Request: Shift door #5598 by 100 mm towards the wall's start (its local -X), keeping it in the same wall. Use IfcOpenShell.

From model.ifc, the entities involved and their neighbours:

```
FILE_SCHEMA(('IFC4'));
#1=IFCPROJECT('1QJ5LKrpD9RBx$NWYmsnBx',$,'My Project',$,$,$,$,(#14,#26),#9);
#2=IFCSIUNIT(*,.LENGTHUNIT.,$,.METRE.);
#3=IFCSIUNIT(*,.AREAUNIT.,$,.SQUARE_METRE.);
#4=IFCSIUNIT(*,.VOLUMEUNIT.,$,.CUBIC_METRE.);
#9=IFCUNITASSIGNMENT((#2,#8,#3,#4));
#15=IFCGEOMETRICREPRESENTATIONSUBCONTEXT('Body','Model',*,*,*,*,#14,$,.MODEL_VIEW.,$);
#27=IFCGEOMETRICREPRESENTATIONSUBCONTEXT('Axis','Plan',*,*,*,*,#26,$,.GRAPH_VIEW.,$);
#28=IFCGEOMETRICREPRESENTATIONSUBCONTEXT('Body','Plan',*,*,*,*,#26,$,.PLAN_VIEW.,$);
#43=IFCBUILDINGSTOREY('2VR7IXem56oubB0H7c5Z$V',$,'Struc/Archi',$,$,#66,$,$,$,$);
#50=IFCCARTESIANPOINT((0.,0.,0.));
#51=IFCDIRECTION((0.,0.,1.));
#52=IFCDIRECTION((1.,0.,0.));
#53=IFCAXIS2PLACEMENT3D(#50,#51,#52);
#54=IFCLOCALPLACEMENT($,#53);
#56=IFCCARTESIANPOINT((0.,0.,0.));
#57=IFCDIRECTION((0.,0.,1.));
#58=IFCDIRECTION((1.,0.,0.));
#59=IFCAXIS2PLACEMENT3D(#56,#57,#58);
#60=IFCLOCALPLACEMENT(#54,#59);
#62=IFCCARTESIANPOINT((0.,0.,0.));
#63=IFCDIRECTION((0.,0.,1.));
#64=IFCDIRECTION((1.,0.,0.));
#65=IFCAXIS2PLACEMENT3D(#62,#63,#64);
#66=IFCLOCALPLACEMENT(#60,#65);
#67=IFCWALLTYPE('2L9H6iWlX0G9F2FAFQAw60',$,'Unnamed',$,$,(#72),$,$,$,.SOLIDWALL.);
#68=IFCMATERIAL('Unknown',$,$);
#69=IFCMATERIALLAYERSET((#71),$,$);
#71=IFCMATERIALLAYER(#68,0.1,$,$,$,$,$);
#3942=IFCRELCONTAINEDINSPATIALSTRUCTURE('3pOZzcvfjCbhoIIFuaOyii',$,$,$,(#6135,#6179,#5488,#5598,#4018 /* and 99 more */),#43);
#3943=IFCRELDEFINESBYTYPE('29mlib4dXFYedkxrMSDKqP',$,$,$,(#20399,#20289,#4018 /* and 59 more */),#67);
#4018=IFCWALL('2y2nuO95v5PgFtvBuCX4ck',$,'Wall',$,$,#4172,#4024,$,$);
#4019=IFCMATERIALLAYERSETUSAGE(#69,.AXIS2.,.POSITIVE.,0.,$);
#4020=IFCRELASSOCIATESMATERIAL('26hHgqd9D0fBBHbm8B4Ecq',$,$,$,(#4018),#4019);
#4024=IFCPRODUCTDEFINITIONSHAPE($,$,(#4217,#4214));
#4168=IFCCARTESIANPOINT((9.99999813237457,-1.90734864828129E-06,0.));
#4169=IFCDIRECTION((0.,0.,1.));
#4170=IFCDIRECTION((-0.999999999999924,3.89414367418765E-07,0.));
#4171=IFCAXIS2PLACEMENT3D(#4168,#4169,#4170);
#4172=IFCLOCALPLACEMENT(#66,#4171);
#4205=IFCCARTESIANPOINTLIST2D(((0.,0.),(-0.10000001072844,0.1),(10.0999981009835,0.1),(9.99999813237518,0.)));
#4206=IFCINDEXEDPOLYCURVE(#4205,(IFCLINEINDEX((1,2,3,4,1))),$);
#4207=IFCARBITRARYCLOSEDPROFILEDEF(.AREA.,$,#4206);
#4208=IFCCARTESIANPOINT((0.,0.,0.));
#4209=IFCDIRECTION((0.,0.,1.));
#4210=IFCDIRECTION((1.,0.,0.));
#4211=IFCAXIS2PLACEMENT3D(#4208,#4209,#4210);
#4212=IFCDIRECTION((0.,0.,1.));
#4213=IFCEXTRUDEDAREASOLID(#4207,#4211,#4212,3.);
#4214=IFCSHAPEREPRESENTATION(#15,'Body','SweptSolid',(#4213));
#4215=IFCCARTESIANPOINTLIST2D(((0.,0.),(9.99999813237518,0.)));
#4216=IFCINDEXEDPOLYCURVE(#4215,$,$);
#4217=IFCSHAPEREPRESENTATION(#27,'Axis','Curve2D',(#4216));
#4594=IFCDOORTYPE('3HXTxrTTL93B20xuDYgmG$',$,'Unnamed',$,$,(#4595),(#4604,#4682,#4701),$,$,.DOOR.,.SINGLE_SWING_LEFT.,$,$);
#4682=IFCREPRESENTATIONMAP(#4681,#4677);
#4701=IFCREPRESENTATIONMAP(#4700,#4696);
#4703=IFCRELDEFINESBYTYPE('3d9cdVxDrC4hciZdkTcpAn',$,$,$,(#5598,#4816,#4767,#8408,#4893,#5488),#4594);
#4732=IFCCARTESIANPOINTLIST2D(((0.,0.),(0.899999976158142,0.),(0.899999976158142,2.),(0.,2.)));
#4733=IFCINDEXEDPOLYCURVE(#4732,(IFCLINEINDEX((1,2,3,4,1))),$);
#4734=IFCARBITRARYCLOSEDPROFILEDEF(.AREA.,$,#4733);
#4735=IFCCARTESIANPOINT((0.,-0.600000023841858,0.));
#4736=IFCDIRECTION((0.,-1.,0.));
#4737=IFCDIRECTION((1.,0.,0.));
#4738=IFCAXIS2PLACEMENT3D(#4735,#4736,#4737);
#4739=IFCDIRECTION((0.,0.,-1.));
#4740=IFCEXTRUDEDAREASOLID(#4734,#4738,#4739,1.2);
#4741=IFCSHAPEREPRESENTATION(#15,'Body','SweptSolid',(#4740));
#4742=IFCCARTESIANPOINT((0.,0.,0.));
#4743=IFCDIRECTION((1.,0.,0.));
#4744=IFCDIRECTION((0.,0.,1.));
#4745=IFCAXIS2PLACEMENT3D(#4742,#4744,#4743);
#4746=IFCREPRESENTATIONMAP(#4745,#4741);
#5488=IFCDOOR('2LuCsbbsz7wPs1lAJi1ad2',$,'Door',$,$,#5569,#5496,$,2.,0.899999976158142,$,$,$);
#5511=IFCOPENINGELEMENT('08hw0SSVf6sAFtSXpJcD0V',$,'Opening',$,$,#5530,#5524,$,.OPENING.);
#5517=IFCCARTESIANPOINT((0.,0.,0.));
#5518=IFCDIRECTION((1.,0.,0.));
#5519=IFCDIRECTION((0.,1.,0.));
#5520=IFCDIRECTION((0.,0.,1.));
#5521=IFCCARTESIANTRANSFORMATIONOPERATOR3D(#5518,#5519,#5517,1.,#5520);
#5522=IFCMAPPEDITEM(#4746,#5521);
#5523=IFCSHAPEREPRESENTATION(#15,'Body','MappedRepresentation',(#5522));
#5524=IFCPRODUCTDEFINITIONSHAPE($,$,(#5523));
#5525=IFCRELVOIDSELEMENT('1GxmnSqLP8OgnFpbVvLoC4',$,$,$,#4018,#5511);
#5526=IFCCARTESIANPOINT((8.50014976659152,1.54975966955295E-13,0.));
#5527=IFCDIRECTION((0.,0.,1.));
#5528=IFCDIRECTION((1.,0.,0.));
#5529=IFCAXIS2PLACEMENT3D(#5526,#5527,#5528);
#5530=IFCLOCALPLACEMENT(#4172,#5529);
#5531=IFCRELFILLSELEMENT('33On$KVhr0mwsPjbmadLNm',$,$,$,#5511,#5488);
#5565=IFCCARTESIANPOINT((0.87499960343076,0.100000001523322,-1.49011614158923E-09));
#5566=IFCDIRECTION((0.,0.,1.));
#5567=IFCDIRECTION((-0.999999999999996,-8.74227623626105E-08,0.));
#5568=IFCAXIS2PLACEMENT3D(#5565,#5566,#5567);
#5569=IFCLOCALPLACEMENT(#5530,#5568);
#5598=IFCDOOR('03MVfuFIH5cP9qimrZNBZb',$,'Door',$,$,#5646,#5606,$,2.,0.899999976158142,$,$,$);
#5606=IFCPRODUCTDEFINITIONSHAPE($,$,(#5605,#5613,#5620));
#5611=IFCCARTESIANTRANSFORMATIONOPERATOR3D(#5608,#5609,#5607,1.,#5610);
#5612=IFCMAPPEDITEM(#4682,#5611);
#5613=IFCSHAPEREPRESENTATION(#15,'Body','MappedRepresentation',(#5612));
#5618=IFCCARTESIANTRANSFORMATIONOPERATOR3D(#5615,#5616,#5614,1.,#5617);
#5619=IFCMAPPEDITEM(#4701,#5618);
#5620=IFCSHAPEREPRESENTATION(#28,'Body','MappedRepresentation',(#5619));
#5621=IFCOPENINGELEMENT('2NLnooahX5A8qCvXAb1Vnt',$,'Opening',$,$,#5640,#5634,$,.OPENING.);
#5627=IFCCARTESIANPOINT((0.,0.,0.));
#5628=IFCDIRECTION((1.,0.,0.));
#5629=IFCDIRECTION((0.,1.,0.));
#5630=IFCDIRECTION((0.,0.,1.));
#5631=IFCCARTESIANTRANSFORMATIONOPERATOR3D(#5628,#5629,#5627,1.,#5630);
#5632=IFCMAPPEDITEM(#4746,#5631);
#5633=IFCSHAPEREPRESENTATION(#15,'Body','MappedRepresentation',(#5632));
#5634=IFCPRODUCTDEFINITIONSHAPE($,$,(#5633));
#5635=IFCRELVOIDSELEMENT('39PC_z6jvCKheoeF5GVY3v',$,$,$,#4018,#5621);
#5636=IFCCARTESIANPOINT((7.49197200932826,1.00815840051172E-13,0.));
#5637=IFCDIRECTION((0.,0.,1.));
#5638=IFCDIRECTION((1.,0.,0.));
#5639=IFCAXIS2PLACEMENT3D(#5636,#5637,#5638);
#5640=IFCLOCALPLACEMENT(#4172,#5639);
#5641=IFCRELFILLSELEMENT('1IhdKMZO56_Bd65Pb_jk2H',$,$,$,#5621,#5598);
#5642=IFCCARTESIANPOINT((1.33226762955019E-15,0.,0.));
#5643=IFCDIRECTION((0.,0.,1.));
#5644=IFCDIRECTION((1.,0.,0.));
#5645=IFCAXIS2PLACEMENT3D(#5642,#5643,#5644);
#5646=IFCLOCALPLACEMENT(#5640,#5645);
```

```python
import ifcopenshell
import ifcopenshell.api.geometry
import ifcopenshell.util.placement
import ifcopenshell.util.unit

model = ifcopenshell.open("model.ifc")
unit_scale = ifcopenshell.util.unit.calculate_unit_scale(model)

door = model.by_guid("03MVfuFIH5cP9qimrZNBZb")
opening = door.FillsVoids[0].RelatingOpeningElement
wall = opening.VoidsElements[0].RelatingBuildingElement

wall_matrix = ifcopenshell.util.placement.get_local_placement(wall.ObjectPlacement)
shift = wall_matrix[:3, 0] * -0.1 / unit_scale
before = ifcopenshell.util.placement.get_local_placement(door.ObjectPlacement)[:3, 3].copy()

# The door is placed relative to its opening, so it follows when the opening moves.
matrix = ifcopenshell.util.placement.get_local_placement(opening.ObjectPlacement)
matrix[:3, 3] += shift
ifcopenshell.api.geometry.edit_object_placement(
    model, product=opening, matrix=matrix, is_si=False, should_transform_children=True
)

after = ifcopenshell.util.placement.get_local_placement(door.ObjectPlacement)[:3, 3]
print("door moved by", (after - before).round(3) + 0.0)

model.write("model_v2.ifc")
```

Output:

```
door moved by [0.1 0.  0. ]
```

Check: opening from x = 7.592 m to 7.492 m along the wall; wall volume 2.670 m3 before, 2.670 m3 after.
